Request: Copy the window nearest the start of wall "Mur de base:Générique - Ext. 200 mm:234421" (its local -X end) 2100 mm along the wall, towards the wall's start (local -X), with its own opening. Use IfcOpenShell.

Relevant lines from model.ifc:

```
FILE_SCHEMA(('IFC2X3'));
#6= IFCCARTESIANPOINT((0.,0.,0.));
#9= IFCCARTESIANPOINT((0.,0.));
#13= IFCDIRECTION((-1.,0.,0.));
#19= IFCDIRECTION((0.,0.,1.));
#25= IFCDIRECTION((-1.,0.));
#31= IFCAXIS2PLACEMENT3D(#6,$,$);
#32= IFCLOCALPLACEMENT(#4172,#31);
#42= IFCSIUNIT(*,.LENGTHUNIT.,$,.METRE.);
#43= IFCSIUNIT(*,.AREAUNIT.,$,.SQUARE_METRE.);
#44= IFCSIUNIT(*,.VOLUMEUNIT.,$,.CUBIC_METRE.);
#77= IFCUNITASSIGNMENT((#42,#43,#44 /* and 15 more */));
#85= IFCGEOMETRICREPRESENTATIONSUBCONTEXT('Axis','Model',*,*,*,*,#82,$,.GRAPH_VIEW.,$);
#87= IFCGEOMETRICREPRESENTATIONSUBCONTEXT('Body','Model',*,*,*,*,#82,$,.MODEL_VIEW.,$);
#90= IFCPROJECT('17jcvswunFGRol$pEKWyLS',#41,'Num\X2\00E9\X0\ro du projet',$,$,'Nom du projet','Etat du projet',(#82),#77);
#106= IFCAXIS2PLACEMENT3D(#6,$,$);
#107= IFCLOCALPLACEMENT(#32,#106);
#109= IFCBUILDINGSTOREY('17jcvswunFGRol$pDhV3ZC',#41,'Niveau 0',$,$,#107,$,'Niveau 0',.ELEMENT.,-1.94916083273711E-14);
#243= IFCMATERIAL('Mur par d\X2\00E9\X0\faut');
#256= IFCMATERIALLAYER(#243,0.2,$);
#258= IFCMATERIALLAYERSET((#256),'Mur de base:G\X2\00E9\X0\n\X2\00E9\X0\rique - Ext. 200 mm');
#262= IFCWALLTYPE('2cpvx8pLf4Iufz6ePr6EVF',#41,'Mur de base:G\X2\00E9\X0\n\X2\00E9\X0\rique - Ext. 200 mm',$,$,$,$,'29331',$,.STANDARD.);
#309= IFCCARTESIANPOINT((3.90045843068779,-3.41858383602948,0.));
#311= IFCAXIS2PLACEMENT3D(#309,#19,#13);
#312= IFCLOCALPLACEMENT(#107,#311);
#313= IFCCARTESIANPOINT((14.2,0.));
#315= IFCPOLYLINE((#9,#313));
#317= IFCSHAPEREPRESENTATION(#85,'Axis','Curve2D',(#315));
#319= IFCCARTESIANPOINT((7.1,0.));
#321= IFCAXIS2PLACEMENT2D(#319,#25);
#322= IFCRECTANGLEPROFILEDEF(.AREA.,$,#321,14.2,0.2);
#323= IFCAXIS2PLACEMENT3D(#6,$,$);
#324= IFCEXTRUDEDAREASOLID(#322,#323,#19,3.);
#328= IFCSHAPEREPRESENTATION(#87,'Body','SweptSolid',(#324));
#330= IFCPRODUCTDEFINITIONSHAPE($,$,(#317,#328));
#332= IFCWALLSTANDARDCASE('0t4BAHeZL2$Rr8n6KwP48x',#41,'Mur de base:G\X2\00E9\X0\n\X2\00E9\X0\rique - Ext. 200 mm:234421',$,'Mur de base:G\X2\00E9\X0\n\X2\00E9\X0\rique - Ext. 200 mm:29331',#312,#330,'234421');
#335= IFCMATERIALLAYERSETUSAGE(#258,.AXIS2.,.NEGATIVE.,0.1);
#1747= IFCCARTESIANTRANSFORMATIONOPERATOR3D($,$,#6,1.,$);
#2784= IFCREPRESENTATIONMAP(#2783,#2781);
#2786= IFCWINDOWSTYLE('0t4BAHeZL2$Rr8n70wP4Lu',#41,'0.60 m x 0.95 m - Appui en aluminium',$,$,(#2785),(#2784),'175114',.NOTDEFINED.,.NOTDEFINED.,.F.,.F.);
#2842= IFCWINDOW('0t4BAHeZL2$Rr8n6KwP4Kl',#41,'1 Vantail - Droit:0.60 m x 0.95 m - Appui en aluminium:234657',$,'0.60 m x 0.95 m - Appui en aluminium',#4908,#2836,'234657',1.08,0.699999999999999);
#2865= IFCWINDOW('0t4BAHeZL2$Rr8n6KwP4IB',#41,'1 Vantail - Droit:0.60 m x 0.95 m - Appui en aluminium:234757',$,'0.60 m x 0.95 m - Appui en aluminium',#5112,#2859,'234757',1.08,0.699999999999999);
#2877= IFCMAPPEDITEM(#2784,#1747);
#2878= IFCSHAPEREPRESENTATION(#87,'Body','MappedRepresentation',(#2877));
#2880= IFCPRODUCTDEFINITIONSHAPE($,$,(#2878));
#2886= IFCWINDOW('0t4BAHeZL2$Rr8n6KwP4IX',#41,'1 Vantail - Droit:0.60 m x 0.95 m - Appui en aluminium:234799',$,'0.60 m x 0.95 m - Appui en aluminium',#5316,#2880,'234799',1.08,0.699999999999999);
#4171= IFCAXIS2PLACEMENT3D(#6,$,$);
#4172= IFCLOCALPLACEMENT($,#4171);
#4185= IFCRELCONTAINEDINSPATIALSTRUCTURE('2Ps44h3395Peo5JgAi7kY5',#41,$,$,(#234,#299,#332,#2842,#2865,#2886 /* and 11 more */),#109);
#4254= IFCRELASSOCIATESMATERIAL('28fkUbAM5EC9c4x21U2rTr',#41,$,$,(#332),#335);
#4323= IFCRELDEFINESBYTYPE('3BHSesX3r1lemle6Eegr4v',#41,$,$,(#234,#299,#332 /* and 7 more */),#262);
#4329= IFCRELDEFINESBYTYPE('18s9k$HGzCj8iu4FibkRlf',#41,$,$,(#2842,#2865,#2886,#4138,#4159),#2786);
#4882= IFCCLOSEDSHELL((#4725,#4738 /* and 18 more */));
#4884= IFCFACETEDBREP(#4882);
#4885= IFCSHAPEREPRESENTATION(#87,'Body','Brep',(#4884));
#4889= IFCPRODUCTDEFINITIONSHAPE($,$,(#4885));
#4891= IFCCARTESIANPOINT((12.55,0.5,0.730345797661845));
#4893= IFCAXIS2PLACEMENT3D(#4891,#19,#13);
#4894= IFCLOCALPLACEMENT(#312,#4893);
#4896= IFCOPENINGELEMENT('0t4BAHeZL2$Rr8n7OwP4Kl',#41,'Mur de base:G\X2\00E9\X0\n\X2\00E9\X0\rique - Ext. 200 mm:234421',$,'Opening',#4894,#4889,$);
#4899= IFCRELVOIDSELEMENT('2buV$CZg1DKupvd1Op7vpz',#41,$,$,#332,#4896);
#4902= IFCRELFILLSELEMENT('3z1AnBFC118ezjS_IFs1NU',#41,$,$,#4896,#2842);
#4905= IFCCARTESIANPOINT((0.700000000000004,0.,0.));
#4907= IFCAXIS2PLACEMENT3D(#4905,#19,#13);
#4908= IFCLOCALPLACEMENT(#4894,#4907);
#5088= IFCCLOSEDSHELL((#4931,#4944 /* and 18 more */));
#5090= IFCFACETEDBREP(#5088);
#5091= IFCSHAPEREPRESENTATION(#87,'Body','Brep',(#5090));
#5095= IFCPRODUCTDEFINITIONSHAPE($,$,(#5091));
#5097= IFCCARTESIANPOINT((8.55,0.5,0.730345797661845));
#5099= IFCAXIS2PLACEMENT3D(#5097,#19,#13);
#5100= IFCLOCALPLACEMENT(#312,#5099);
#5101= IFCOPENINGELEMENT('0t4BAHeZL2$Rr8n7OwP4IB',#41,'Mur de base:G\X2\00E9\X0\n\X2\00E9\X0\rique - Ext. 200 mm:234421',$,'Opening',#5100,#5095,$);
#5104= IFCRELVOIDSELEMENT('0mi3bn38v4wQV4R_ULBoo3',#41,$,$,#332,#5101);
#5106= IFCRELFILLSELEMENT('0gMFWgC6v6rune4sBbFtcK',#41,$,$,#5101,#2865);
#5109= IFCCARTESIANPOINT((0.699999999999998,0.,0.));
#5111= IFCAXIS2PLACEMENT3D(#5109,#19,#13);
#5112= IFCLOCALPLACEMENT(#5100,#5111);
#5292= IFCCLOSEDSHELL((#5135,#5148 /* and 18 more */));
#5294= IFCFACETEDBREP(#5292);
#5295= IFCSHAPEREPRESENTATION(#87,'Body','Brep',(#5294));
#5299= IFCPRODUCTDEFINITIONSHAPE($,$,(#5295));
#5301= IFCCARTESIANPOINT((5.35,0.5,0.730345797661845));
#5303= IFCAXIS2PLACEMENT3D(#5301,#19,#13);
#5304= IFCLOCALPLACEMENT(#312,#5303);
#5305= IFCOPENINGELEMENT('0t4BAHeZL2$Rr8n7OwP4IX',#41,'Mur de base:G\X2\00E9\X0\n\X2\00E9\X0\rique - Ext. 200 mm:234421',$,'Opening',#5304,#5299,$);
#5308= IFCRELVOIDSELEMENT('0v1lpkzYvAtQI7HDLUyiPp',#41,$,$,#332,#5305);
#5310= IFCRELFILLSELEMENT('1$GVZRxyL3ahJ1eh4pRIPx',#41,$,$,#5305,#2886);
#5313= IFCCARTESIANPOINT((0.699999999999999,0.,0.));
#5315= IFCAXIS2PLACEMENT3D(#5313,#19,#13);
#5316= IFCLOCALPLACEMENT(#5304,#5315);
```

```python
import ifcopenshell
import ifcopenshell.api.feature
import ifcopenshell.api.geometry
import ifcopenshell.api.root
import ifcopenshell.geom
import ifcopenshell.util.element
import ifcopenshell.util.placement
import ifcopenshell.util.shape
import ifcopenshell.util.unit

model = ifcopenshell.open("model.ifc")
unit_scale = ifcopenshell.util.unit.calculate_unit_scale(model)
settings = ifcopenshell.geom.settings()


def volume(element):
    """Net volume in cubic metres, openings subtracted."""
    shape = ifcopenshell.geom.create_shape(settings, element)
    return ifcopenshell.util.shape.get_volume(shape.geometry)


def reuse_history(source, copy):
    """copy_class also copies each property set's owner history, people and application; keep the originals."""
    for rel in copy.IsDefinedBy:
        if rel.is_a("IfcRelDefinesByProperties") and (history := rel.RelatingPropertyDefinition.OwnerHistory):
            rel.RelatingPropertyDefinition.OwnerHistory = source.OwnerHistory
            ifcopenshell.util.element.remove_deep2(model, history)


window = model.by_guid("0t4BAHeZL2$Rr8n6KwP4IX")
opening = window.FillsVoids[0].RelatingOpeningElement
wall = opening.VoidsElements[0].RelatingBuildingElement
before = volume(wall)
shift = ifcopenshell.util.placement.get_local_placement(wall.ObjectPlacement)[:3, 0] * -2.1 / unit_scale

# copy_class copies the void relationship, type, container and properties, but no geometry.
new_opening = ifcopenshell.api.root.copy_class(model, product=opening)
new_opening.Representation = ifcopenshell.util.element.copy_deep(
    model, opening.Representation, exclude=["IfcGeometricRepresentationContext", "IfcRepresentationMap"]
)
new_opening.Name = "Mur de base:Générique - Ext. 200 mm"
new_window = ifcopenshell.api.root.copy_class(model, product=window)
new_window.Representation = ifcopenshell.util.element.copy_deep(
    model, window.Representation, exclude=["IfcGeometricRepresentationContext", "IfcRepresentationMap"]
)
new_window.Name = "1 Vantail - Droit:0.60 m x 0.95 m - Appui en aluminium"
new_window.Tag = None
reuse_history(window, new_window)
fills = ifcopenshell.api.feature.add_filling(model, opening=new_opening, element=new_window)
fills.OwnerHistory = new_window.OwnerHistory  # required in IFC2X3

for old, new in ((opening, new_opening), (window, new_window)):
    matrix = ifcopenshell.util.placement.get_local_placement(old.ObjectPlacement)
    matrix[:3, 3] += shift
    ifcopenshell.api.geometry.edit_object_placement(model, product=new, matrix=matrix, is_si=False)

after = volume(wall)

print(f"wall volume {before:.3f} -> {after:.3f} m3")

model.write("model-out.ifc")
```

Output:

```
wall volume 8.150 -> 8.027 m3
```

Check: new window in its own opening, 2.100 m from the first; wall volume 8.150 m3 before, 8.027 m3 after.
